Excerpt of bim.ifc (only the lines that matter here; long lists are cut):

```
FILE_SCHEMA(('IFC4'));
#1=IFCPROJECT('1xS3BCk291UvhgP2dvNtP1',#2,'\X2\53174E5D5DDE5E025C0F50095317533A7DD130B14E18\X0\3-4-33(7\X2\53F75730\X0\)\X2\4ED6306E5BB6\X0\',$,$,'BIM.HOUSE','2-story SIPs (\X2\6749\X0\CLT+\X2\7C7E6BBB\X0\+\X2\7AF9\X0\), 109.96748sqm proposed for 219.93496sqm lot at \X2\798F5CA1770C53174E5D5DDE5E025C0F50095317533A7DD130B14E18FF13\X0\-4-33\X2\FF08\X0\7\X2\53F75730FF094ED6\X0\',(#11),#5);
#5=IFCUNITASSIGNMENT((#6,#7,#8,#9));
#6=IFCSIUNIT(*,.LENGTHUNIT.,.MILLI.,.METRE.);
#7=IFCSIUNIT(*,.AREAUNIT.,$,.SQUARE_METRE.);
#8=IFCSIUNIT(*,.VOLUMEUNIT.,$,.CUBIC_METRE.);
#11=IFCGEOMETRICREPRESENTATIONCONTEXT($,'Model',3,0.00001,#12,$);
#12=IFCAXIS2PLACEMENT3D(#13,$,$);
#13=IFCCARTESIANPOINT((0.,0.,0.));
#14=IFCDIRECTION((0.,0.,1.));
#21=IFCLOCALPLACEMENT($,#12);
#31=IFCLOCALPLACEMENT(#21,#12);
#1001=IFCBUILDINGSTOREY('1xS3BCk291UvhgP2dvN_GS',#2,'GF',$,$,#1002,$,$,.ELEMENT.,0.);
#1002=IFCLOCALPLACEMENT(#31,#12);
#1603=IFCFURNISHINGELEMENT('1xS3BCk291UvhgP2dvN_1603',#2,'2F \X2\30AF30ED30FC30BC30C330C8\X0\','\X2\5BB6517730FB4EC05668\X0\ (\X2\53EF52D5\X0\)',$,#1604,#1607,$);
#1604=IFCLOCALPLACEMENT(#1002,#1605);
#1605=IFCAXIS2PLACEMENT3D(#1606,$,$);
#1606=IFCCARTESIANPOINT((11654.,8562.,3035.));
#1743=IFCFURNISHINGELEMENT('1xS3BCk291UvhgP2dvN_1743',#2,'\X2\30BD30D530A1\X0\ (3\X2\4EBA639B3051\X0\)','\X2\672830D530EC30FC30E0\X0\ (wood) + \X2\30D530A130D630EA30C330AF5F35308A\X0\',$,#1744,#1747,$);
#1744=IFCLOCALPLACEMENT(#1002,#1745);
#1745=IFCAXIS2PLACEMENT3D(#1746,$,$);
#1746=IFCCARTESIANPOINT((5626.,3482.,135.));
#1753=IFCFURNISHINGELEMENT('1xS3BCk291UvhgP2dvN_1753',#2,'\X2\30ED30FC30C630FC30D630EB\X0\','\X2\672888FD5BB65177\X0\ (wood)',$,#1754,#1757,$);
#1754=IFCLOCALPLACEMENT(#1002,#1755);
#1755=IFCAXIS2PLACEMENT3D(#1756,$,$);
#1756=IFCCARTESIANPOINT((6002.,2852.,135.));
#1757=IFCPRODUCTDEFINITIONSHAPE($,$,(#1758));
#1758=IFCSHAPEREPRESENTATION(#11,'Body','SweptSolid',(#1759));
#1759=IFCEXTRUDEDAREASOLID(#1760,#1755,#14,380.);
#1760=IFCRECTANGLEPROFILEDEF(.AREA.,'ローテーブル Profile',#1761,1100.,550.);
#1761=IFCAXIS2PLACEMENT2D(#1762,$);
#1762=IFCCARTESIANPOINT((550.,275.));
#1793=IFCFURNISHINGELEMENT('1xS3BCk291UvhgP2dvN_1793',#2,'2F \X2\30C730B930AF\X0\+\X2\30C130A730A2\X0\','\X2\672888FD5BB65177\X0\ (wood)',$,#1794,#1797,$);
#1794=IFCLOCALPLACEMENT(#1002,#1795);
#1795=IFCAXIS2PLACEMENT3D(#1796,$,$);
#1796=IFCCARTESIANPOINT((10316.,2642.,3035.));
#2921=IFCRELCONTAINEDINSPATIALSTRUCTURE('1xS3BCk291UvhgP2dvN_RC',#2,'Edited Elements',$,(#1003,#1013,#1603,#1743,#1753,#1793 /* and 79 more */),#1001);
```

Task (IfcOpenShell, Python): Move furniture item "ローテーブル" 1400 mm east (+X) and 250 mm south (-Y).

```python
import ifcopenshell
import ifcopenshell.api.geometry
import ifcopenshell.util.placement

model = ifcopenshell.open("bim.ifc")

item = model.by_id(1753)
matrix = ifcopenshell.util.placement.get_local_placement(item.ObjectPlacement)
matrix[0, 3] += 1400.0
matrix[1, 3] -= 250.0
ifcopenshell.api.geometry.edit_object_placement(model, product=item, matrix=matrix, is_si=False)

print(ifcopenshell.util.placement.get_local_placement(item.ObjectPlacement).round(3) + 0.0)

model.write("bim-out.ifc")
```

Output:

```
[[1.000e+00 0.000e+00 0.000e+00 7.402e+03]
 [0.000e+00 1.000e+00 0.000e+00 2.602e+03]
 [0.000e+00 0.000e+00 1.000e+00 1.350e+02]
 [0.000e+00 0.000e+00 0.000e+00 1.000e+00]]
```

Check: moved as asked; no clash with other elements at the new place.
